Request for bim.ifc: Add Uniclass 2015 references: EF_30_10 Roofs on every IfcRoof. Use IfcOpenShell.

First a look at what the model holds.

```python
import ifcopenshell

model = ifcopenshell.open("bim.ifc")
print(model.schema)
print("classifications:", [c.Name for c in model.by_type("IfcClassification")])
for ifc_class in ("IfcDoor", "IfcRoof", "IfcStair", "IfcWall", "IfcWindow"):
    print(ifc_class, len(model.by_type(ifc_class)))
```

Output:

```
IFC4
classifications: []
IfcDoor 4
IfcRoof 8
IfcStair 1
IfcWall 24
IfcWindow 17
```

```python
import ifcopenshell
import ifcopenshell.api.classification

model = ifcopenshell.open("bim.ifc")

system = ifcopenshell.api.classification.add_classification(model, classification="Uniclass 2015")

codes = {
    "IfcRoof": ("EF_30_10", "Roofs"),
}
for ifc_class, (code, name) in codes.items():
    products = model.by_type(ifc_class)
    ifcopenshell.api.classification.add_reference(
        model, products=products, classification=system, identification=code, name=name
    )
    print(code, len(products))

model.write("bim_rev.ifc")
```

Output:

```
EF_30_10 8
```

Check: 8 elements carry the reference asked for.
